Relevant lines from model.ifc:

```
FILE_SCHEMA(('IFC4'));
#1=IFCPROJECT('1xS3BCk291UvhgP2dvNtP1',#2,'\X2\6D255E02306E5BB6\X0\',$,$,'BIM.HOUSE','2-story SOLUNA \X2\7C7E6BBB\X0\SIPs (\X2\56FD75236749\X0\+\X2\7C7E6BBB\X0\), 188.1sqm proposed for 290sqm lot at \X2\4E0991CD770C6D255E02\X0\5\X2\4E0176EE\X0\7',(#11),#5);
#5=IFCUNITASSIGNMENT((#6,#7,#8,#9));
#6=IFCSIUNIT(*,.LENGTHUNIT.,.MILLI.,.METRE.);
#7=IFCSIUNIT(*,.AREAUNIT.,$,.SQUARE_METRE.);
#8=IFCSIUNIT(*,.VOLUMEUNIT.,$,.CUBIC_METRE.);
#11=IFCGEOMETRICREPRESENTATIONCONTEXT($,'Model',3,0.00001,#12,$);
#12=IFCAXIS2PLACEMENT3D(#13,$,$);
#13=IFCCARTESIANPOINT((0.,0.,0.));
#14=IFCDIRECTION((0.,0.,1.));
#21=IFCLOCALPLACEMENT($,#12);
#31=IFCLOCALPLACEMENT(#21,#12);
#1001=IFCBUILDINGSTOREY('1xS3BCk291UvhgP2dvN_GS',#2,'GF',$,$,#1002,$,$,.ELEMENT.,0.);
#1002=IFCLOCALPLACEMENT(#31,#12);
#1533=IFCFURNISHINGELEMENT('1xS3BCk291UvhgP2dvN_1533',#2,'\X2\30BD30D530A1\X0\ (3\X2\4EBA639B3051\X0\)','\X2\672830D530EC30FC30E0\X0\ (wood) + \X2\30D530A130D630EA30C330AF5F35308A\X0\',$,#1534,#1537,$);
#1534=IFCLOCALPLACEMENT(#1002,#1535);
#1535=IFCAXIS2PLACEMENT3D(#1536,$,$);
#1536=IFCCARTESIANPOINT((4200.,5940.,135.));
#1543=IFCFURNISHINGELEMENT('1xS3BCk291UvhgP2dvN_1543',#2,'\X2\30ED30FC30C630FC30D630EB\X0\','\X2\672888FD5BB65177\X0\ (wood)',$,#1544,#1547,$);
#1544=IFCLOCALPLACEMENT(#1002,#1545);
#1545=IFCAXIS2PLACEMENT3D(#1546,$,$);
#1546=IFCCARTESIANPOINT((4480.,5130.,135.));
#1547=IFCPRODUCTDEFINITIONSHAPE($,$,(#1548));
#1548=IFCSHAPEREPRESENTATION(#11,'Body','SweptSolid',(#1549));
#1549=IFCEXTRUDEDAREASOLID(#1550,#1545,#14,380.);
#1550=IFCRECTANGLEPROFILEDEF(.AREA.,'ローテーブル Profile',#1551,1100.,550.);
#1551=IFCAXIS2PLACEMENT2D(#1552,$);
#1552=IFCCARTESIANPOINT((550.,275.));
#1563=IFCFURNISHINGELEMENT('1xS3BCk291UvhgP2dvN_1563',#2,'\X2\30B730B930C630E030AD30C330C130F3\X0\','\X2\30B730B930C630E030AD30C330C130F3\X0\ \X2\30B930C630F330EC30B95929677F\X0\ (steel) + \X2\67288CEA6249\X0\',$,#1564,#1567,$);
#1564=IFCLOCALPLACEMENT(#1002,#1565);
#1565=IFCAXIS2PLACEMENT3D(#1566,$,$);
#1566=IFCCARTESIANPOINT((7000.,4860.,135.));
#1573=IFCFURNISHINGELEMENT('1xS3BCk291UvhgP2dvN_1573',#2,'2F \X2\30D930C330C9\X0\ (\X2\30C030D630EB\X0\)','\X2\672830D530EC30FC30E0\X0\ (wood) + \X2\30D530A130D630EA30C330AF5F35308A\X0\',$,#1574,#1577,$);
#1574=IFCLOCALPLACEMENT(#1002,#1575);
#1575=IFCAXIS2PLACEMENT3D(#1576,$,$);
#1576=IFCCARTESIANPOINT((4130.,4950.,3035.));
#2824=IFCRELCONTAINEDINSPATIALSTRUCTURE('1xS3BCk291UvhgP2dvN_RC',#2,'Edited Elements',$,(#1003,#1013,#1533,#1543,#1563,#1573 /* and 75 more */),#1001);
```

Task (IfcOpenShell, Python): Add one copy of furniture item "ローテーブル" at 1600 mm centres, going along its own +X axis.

```python
import ifcopenshell
import ifcopenshell.api.geometry
import ifcopenshell.api.root
import ifcopenshell.util.element
import ifcopenshell.util.placement
import ifcopenshell.util.unit

model = ifcopenshell.open("model.ifc")
unit_scale = ifcopenshell.util.unit.calculate_unit_scale(model)


def reuse_history(source, copy):
    """copy_class also copies each property set's owner history, people and application; keep the originals."""
    for rel in copy.IsDefinedBy:
        if rel.is_a("IfcRelDefinesByProperties") and (history := rel.RelatingPropertyDefinition.OwnerHistory):
            rel.RelatingPropertyDefinition.OwnerHistory = source.OwnerHistory
            ifcopenshell.util.element.remove_deep2(model, history)


source = model.by_guid("1xS3BCk291UvhgP2dvN_1543")
base = ifcopenshell.util.placement.get_local_placement(source.ObjectPlacement)
step = base[:3, 0] * 1.6 / unit_scale

for i in range(1, 2):
    copy = ifcopenshell.api.root.copy_class(model, product=source)
    copy.Representation = ifcopenshell.util.element.copy_deep(
        model, source.Representation, exclude=["IfcGeometricRepresentationContext", "IfcRepresentationMap"]
    )
    reuse_history(source, copy)
    matrix = base.copy()
    matrix[:3, 3] += i * step
    print("added at", matrix[:3, 3].round(3) + 0.0)
    ifcopenshell.api.geometry.edit_object_placement(model, product=copy, matrix=matrix, is_si=False)

model.write("model_v2.ifc")
```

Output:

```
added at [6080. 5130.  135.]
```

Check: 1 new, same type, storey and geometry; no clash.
